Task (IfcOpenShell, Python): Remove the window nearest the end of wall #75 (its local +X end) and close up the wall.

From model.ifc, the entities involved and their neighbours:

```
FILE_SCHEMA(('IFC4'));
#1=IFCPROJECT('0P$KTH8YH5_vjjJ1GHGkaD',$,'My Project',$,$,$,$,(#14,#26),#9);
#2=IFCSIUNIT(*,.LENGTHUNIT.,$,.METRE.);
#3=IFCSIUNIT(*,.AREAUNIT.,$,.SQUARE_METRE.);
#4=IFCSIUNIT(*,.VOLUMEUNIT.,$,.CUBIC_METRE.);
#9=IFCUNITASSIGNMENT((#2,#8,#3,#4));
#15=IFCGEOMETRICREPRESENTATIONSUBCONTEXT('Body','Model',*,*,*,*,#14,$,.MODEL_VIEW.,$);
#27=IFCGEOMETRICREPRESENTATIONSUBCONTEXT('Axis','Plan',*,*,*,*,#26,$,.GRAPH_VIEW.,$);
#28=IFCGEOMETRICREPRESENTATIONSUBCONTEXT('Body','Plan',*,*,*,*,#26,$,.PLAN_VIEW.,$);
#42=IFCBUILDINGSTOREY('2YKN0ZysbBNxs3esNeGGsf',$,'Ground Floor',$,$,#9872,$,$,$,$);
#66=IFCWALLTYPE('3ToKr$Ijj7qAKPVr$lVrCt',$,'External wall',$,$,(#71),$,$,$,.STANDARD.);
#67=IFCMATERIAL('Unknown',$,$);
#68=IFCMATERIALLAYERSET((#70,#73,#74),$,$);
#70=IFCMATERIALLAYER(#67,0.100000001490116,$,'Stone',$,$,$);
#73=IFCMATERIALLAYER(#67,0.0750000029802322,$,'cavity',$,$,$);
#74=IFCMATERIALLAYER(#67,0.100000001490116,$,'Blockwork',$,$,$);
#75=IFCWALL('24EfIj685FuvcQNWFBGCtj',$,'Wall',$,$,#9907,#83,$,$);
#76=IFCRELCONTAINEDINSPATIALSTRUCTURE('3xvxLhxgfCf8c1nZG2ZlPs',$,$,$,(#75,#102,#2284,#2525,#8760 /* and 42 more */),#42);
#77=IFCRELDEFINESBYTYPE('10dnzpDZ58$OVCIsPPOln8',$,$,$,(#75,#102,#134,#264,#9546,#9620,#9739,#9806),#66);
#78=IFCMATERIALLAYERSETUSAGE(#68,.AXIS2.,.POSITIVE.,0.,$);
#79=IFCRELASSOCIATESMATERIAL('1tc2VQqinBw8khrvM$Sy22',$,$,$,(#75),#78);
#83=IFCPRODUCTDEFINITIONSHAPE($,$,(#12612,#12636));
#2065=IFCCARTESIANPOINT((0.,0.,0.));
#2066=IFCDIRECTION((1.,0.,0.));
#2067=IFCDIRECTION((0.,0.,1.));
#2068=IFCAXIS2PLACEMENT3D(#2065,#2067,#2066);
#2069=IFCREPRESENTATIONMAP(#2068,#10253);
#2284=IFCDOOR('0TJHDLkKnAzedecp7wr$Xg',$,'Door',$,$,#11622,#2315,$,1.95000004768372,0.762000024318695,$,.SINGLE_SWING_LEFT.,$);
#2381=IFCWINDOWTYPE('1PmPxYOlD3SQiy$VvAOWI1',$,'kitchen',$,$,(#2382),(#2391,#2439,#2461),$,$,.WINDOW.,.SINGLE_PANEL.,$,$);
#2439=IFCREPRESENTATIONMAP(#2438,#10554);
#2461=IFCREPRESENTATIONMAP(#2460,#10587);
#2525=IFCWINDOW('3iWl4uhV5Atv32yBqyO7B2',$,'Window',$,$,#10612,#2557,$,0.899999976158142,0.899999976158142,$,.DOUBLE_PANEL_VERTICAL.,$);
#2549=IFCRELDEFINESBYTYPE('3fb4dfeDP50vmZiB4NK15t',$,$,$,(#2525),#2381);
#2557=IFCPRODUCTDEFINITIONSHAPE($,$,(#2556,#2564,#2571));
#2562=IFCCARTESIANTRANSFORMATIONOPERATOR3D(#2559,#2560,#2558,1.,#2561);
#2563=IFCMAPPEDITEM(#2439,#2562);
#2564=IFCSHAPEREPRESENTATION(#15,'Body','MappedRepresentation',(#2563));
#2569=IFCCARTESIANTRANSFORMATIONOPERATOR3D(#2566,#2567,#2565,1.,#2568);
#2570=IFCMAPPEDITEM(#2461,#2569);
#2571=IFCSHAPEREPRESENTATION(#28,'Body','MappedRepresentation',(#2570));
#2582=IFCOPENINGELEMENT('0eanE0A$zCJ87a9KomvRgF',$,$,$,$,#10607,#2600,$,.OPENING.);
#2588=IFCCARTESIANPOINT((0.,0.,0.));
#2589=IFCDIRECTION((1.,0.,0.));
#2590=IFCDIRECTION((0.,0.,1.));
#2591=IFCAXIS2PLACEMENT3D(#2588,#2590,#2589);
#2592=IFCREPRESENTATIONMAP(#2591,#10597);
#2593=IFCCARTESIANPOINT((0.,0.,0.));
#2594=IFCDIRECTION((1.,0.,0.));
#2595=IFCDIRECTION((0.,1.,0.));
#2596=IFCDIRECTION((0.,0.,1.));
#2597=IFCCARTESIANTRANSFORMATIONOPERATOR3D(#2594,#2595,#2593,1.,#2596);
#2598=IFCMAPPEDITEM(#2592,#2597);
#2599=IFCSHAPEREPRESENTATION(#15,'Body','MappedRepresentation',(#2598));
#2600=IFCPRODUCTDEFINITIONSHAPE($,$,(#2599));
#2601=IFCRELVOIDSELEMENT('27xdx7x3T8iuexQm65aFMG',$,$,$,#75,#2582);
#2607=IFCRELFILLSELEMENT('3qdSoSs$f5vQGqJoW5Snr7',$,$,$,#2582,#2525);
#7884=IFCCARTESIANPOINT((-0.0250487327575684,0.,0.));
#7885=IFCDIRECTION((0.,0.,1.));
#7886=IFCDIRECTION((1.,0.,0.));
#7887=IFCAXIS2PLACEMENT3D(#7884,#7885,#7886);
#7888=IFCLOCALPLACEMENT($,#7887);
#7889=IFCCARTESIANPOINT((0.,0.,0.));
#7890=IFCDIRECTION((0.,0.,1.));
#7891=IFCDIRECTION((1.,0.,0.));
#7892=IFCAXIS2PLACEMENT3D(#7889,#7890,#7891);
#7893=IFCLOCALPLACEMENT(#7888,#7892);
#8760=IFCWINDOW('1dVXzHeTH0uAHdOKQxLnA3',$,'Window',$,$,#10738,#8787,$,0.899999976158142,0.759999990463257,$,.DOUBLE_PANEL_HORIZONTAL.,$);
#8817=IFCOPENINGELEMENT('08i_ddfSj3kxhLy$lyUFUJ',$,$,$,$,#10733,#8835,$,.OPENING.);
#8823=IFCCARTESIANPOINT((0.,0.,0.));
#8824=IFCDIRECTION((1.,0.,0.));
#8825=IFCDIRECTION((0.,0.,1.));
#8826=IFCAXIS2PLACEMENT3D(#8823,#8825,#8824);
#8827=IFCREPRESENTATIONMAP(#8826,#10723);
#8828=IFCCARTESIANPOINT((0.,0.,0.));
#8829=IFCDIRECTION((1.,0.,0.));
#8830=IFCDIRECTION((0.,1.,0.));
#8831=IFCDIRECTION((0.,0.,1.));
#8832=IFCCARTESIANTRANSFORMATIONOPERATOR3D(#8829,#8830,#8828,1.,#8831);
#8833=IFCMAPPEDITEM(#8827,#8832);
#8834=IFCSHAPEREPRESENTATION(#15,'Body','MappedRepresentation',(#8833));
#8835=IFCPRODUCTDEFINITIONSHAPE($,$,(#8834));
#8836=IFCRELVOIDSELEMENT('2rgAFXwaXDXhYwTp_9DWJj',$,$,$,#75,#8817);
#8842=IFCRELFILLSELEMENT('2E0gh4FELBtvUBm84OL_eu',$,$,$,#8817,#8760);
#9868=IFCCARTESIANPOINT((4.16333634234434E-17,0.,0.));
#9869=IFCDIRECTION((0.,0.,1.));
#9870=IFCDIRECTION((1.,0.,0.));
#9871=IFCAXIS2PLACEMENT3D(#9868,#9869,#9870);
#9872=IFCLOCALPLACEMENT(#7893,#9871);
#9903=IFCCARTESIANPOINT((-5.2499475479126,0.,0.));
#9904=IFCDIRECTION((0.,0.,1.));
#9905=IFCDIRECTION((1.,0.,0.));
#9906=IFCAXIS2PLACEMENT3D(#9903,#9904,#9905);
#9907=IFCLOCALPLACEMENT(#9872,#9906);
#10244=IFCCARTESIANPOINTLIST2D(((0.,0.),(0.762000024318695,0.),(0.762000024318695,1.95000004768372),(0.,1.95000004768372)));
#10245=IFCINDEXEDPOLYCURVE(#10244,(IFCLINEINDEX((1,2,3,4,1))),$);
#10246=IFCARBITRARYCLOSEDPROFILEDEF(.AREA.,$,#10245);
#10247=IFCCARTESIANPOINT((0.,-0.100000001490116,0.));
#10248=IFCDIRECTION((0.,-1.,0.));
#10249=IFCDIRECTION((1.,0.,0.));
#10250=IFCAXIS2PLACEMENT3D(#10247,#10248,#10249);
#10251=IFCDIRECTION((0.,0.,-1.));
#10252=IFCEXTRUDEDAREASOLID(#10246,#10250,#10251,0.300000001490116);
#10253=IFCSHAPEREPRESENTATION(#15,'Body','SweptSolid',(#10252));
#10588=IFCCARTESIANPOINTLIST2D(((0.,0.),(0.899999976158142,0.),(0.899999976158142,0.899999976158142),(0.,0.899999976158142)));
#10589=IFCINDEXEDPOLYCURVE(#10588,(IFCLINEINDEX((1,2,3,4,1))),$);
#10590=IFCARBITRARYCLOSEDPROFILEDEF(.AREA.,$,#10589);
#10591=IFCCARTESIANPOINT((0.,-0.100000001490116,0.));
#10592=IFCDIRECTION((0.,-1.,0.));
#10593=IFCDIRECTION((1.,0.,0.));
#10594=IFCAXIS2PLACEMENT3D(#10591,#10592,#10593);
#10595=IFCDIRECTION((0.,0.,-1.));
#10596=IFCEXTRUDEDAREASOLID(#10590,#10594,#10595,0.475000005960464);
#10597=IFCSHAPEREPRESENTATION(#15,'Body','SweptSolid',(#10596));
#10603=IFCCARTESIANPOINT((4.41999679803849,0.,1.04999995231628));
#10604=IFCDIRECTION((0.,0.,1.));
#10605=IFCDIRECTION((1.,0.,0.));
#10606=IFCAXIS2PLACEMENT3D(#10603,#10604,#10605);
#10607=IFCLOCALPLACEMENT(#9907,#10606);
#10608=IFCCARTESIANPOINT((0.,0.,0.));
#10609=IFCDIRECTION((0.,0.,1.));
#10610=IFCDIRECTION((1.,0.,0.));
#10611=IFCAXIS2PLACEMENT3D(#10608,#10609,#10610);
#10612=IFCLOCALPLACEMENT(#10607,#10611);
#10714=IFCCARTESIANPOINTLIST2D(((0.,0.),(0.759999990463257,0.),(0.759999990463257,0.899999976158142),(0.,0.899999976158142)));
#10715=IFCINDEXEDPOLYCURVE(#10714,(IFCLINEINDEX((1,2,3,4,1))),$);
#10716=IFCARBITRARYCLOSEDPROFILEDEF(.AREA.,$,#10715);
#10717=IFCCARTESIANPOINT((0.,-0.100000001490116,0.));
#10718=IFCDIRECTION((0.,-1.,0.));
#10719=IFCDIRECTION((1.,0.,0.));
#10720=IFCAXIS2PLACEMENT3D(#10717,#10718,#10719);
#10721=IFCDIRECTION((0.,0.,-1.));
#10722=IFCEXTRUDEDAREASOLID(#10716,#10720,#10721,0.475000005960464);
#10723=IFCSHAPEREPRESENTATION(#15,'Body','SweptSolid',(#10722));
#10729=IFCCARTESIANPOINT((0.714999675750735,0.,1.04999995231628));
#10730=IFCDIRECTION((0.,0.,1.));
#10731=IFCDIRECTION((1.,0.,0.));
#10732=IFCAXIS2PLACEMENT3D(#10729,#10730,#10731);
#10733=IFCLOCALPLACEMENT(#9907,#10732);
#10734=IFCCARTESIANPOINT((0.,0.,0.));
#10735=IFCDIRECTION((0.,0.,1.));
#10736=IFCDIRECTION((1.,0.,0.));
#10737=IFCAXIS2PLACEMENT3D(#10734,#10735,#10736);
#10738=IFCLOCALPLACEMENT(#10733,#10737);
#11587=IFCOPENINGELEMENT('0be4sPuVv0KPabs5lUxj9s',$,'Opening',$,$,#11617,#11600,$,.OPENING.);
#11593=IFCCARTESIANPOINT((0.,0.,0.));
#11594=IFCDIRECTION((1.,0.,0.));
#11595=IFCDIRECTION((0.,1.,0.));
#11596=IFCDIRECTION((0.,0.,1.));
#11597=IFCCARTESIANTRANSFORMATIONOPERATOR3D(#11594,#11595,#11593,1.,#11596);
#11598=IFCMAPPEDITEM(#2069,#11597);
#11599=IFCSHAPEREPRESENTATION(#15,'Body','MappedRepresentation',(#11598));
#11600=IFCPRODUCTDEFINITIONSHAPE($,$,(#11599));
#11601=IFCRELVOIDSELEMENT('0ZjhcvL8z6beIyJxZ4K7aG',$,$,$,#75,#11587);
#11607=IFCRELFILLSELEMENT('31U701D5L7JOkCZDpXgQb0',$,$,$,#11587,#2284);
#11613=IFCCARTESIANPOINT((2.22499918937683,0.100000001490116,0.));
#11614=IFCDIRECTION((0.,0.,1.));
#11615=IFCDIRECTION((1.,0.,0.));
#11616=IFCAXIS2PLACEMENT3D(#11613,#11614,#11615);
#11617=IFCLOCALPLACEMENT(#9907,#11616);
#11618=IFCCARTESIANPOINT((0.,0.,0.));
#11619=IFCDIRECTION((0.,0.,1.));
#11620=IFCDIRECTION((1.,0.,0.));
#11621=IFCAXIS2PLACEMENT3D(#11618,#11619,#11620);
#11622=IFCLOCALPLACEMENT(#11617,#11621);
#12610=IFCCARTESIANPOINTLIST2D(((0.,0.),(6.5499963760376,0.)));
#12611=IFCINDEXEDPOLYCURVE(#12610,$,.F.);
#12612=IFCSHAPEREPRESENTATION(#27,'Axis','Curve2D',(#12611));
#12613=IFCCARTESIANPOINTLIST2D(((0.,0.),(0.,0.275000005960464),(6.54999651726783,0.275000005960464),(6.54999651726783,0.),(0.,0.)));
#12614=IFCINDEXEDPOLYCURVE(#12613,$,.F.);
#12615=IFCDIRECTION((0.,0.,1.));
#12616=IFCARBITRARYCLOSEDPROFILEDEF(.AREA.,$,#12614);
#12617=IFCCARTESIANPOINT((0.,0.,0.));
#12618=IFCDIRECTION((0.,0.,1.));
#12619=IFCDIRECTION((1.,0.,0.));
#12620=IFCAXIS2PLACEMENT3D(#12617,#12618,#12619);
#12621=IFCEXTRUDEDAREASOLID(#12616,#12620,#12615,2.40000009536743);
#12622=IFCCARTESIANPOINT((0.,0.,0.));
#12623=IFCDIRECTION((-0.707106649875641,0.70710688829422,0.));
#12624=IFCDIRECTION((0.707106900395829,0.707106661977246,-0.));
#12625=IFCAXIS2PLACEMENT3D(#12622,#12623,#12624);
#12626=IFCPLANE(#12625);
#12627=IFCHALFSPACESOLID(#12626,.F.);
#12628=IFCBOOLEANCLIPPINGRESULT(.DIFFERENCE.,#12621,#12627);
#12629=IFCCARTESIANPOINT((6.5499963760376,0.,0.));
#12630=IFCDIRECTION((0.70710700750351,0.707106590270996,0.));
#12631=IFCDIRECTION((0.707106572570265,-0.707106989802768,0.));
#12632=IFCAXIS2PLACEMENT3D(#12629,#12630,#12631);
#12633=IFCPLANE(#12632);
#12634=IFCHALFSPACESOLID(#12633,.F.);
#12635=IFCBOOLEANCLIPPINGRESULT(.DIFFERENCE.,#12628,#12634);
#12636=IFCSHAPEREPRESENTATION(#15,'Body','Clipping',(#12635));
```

```python
import ifcopenshell
import ifcopenshell.api.feature
import ifcopenshell.api.root
import ifcopenshell.geom
import ifcopenshell.util.shape

model = ifcopenshell.open("model.ifc")
settings = ifcopenshell.geom.settings()


def volume(element):
    """Net volume in cubic metres, openings subtracted."""
    shape = ifcopenshell.geom.create_shape(settings, element)
    return ifcopenshell.util.shape.get_volume(shape.geometry)


window = model.by_guid("3iWl4uhV5Atv32yBqyO7B2")
opening = window.FillsVoids[0].RelatingOpeningElement
wall = opening.VoidsElements[0].RelatingBuildingElement
before = volume(wall)

ifcopenshell.api.root.remove_product(model, product=window)
ifcopenshell.api.feature.remove_feature(model, feature=opening)

after = volume(wall)

print(f"wall volume {before:.3f} -> {after:.3f} m3")

model.write("model_edited.ifc")
```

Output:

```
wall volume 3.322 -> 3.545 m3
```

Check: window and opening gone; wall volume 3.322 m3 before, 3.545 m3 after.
